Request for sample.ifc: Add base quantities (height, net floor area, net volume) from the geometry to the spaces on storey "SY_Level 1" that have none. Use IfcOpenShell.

First a look at what the model holds.

```python
import ifcopenshell
import ifcopenshell.util.element
import ifcopenshell.util.unit

model = ifcopenshell.open("sample.ifc")
print(model.schema)
for unit_type in ("LENGTHUNIT", "AREAUNIT", "VOLUMEUNIT"):
    print(unit_type, ifcopenshell.util.unit.calculate_unit_scale(model, unit_type))
storey = next(s for s in model.by_type("IfcBuildingStorey") if s.Name == "SY_Level 1")
spaces = [e for e in ifcopenshell.util.element.get_decomposition(storey) if e.is_a("IfcSpace")]
for e in sorted(spaces, key=lambda e: e.id()):
    print(e.id(), e.is_a(), e.Name, list(ifcopenshell.util.element.get_psets(e, qtos_only=True)), sep=" | ")
```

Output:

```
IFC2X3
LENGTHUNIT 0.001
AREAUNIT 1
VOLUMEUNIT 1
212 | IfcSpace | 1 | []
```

```python
import ifcopenshell
import ifcopenshell.api.pset
import ifcopenshell.geom
import ifcopenshell.util.element
import ifcopenshell.util.shape
import ifcopenshell.util.unit

model = ifcopenshell.open("sample.ifc")
unit_scale = ifcopenshell.util.unit.calculate_unit_scale(model)
area_scale = ifcopenshell.util.unit.calculate_unit_scale(model, "AREAUNIT")
volume_scale = ifcopenshell.util.unit.calculate_unit_scale(model, "VOLUMEUNIT")
settings = ifcopenshell.geom.settings()

storey = next(s for s in model.by_type("IfcBuildingStorey") if s.Name == "SY_Level 1")
spaces = [e for e in ifcopenshell.util.element.get_decomposition(storey) if e.is_a("IfcSpace")]

for e in sorted(spaces, key=lambda e: e.id()):
    if ifcopenshell.util.element.get_psets(e, qtos_only=True, should_inherit=False):
        continue
    # Geometry comes back in metres, in the element's own axes.
    shape = ifcopenshell.geom.create_shape(settings, e)
    values = {
        "Height": ifcopenshell.util.shape.get_z(shape.geometry) / unit_scale,
        "NetFloorArea": ifcopenshell.util.shape.get_footprint_area(shape.geometry) / area_scale,
        "NetVolume": ifcopenshell.util.shape.get_volume(shape.geometry) / volume_scale,
    }
    qto = ifcopenshell.api.pset.add_qto(model, product=e, name="BaseQuantities")
    ifcopenshell.api.pset.edit_qto(model, qto=qto, properties=values)
    print(e.id(), {k: round(v, 3) for k, v in values.items()})

model.write("sample-out.ifc")
```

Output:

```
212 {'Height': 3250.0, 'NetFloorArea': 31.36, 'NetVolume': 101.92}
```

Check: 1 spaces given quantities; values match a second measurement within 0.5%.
